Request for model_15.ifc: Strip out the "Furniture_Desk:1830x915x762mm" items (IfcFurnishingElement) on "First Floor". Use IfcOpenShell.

First a look at what the model holds.

```python
import ifcopenshell
import ifcopenshell.util.element

model = ifcopenshell.open("model_15.ifc")
print(model.schema)
storey = next(s for s in model.by_type("IfcBuildingStorey") if s.Name == "First Floor")
furniture = [e for e in ifcopenshell.util.element.get_decomposition(storey) if e.is_a("IfcFurnishingElement")]
seen = {}
for e in furniture:
    element_type = ifcopenshell.util.element.get_type(e)
    name = element_type.Name if element_type not in (None, e) else None
    seen[name] = seen.get(name, 0) + 1
for name, count in sorted(seen.items(), key=str):
    print(count, "x", name)
```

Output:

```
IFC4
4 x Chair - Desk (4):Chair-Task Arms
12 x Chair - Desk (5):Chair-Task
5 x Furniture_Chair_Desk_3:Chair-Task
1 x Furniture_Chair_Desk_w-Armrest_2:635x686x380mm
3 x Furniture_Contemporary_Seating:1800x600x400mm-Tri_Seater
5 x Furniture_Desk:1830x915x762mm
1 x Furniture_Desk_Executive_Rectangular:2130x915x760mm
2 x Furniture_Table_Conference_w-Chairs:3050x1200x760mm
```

```python
import ifcopenshell
import ifcopenshell.api.root
import ifcopenshell.util.element

model = ifcopenshell.open("model_15.ifc")

storey = next(s for s in model.by_type("IfcBuildingStorey") if s.Name == "First Floor")
furniture = [e for e in ifcopenshell.util.element.get_decomposition(storey) if e.is_a("IfcFurnishingElement")]
targets = [e for e in furniture if (t := ifcopenshell.util.element.get_type(e)) not in (None, e) and t.Name == "Furniture_Desk:1830x915x762mm"]

for e in targets:
    ifcopenshell.api.root.remove_product(model, product=e)
print(len(targets), "removed")

model.write("model_15-out.ifc")
```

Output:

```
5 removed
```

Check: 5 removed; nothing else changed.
